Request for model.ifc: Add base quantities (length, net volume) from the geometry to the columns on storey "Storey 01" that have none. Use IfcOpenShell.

First a look at what the model holds.

```python
import ifcopenshell
import ifcopenshell.util.element
import ifcopenshell.util.unit

model = ifcopenshell.open("model.ifc")
print(model.schema)
for unit_type in ("LENGTHUNIT", "AREAUNIT", "VOLUMEUNIT"):
    print(unit_type, ifcopenshell.util.unit.calculate_unit_scale(model, unit_type))
storey = next(s for s in model.by_type("IfcBuildingStorey") if s.Name == "Storey 01")
columns = [e for e in ifcopenshell.util.element.get_decomposition(storey) if e.is_a("IfcColumn")]
for e in sorted(columns, key=lambda e: e.id()):
    print(e.id(), e.is_a(), e.Name, list(ifcopenshell.util.element.get_psets(e, qtos_only=True)), sep=" | ")
```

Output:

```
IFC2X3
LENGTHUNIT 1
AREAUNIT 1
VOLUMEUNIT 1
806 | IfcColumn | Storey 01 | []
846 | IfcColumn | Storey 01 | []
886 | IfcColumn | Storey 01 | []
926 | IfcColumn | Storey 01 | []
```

```python
import ifcopenshell
import ifcopenshell.api.pset
import ifcopenshell.geom
import ifcopenshell.util.element
import ifcopenshell.util.shape
import ifcopenshell.util.unit

model = ifcopenshell.open("model.ifc")
unit_scale = ifcopenshell.util.unit.calculate_unit_scale(model)
volume_scale = ifcopenshell.util.unit.calculate_unit_scale(model, "VOLUMEUNIT")
settings = ifcopenshell.geom.settings()

storey = next(s for s in model.by_type("IfcBuildingStorey") if s.Name == "Storey 01")
columns = [e for e in ifcopenshell.util.element.get_decomposition(storey) if e.is_a("IfcColumn")]

for e in sorted(columns, key=lambda e: e.id()):
    if ifcopenshell.util.element.get_psets(e, qtos_only=True, should_inherit=False):
        continue
    # Geometry comes back in metres, in the element's own axes.
    shape = ifcopenshell.geom.create_shape(settings, e)
    values = {
        "Length": ifcopenshell.util.shape.get_z(shape.geometry) / unit_scale,
        "NetVolume": ifcopenshell.util.shape.get_volume(shape.geometry) / volume_scale,
    }
    qto = ifcopenshell.api.pset.add_qto(model, product=e, name="BaseQuantities")
    ifcopenshell.api.pset.edit_qto(model, qto=qto, properties=values)
    print(e.id(), {k: round(v, 3) for k, v in values.items()})

model.write("model_edited.ifc")
```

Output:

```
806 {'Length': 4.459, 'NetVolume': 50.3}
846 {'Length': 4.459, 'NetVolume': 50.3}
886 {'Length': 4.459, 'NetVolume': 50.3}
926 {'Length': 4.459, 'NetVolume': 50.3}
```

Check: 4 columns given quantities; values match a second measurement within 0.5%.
